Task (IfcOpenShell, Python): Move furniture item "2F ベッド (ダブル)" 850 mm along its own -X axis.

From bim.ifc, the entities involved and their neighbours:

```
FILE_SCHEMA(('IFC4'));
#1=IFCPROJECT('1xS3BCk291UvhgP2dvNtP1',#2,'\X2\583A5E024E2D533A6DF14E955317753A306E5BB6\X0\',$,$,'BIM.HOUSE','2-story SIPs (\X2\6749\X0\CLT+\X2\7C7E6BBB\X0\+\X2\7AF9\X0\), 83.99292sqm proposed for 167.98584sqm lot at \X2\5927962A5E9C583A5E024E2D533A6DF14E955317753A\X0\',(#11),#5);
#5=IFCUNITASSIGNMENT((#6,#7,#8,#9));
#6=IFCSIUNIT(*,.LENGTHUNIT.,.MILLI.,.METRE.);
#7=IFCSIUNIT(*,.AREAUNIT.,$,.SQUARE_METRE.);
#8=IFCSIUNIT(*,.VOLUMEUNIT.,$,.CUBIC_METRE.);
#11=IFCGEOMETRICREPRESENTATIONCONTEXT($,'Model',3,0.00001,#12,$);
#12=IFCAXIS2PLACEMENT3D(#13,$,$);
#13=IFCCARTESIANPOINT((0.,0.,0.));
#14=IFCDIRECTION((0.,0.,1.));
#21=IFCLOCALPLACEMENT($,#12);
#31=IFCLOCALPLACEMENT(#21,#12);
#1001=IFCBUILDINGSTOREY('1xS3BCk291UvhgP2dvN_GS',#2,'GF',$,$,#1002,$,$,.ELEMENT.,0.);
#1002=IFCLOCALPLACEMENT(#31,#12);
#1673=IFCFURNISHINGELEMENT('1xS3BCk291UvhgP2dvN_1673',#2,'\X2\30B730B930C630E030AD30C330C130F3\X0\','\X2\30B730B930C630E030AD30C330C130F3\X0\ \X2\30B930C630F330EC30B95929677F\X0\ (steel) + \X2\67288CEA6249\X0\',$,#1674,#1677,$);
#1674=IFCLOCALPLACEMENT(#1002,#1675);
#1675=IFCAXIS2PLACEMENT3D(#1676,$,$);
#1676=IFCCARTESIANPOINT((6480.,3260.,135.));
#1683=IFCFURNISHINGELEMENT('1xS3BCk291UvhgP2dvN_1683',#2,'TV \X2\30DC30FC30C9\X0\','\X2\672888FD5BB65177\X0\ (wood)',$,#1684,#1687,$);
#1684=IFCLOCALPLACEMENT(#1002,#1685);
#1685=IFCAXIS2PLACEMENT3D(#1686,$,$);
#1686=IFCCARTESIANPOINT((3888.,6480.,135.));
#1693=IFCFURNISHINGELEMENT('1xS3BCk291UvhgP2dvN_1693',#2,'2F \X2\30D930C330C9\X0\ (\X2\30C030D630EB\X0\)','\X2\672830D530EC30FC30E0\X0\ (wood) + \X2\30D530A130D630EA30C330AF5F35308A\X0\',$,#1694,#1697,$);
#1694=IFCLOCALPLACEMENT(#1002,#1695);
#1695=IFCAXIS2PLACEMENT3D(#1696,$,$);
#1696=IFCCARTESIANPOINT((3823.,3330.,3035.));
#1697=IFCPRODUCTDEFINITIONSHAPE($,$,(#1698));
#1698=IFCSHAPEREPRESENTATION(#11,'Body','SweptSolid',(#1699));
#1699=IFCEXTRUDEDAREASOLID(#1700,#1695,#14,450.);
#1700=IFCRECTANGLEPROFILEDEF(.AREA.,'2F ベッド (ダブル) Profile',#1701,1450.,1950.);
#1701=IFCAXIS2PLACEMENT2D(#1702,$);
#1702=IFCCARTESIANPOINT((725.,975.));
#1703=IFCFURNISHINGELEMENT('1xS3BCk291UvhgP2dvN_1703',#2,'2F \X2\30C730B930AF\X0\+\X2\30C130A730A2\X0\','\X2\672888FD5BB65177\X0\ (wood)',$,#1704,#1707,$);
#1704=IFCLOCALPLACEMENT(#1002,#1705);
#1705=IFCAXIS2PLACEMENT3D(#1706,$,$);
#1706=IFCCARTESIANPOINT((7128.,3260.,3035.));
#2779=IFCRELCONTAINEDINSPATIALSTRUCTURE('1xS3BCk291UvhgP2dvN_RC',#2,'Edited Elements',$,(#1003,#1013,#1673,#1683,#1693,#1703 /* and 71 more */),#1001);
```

```python
import ifcopenshell
import ifcopenshell.api.geometry
import ifcopenshell.util.placement
import ifcopenshell.util.unit

model = ifcopenshell.open("bim.ifc")
unit_scale = ifcopenshell.util.unit.calculate_unit_scale(model)

item = model.by_id(1693)
matrix = ifcopenshell.util.placement.get_local_placement(item.ObjectPlacement)
matrix[:3, 3] -= matrix[:3, 0] * 0.85 / unit_scale
ifcopenshell.api.geometry.edit_object_placement(model, product=item, matrix=matrix, is_si=False)

print(ifcopenshell.util.placement.get_local_placement(item.ObjectPlacement).round(3) + 0.0)

model.write("bim-out.ifc")
```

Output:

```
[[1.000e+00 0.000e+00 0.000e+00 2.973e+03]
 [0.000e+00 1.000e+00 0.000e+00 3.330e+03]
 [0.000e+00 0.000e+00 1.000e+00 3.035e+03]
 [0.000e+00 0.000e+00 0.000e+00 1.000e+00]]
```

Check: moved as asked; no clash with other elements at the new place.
